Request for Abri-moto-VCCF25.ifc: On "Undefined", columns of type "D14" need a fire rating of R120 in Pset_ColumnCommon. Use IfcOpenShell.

First a look at what the model holds.

```python
import ifcopenshell
import ifcopenshell.util.element

model = ifcopenshell.open("Abri-moto-VCCF25.ifc")
print(model.schema)
storey = next(s for s in model.by_type("IfcBuildingStorey") if s.Name == "Undefined")
columns = [e for e in ifcopenshell.util.element.get_decomposition(storey) if e.is_a("IfcColumn")]
seen = {}
for e in columns:
    element_type = ifcopenshell.util.element.get_type(e)
    key = (element_type.Name if element_type != e and element_type else None, ifcopenshell.util.element.get_pset(e, "Pset_ColumnCommon", "FireRating"))
    seen[key] = seen.get(key, 0) + 1
for (name, value), count in sorted(seen.items(), key=str):
    print(count, "x", name, "|", value)
```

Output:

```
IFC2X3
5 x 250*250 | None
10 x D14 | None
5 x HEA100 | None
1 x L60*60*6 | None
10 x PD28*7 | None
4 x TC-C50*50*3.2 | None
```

```python
import ifcopenshell
import ifcopenshell.api.pset
import ifcopenshell.util.element

model = ifcopenshell.open("Abri-moto-VCCF25.ifc")

storey = next(s for s in model.by_type("IfcBuildingStorey") if s.Name == "Undefined")
columns = [e for e in ifcopenshell.util.element.get_decomposition(storey) if e.is_a("IfcColumn")]

count = 0
for e in columns:
    element_type = ifcopenshell.util.element.get_type(e)
    if element_type in (None, e) or element_type.Name != "D14":
        continue
    found = ifcopenshell.util.element.get_pset(e, "Pset_ColumnCommon", should_inherit=False)
    if found:
        pset = model.by_id(found["id"])
        if len(ifcopenshell.util.element.get_elements_by_pset(pset)) > 1:
            pset = ifcopenshell.api.pset.unshare_pset(model, products=[e], pset=pset)[0]
    else:
        pset = ifcopenshell.api.pset.add_pset(model, product=e, name="Pset_ColumnCommon")
    ifcopenshell.api.pset.edit_pset(model, pset=pset, properties={"FireRating": "R120"})
    count += 1

print(count, "columns updated")

model.write("Abri-moto-VCCF25-out.ifc")
```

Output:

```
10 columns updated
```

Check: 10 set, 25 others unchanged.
